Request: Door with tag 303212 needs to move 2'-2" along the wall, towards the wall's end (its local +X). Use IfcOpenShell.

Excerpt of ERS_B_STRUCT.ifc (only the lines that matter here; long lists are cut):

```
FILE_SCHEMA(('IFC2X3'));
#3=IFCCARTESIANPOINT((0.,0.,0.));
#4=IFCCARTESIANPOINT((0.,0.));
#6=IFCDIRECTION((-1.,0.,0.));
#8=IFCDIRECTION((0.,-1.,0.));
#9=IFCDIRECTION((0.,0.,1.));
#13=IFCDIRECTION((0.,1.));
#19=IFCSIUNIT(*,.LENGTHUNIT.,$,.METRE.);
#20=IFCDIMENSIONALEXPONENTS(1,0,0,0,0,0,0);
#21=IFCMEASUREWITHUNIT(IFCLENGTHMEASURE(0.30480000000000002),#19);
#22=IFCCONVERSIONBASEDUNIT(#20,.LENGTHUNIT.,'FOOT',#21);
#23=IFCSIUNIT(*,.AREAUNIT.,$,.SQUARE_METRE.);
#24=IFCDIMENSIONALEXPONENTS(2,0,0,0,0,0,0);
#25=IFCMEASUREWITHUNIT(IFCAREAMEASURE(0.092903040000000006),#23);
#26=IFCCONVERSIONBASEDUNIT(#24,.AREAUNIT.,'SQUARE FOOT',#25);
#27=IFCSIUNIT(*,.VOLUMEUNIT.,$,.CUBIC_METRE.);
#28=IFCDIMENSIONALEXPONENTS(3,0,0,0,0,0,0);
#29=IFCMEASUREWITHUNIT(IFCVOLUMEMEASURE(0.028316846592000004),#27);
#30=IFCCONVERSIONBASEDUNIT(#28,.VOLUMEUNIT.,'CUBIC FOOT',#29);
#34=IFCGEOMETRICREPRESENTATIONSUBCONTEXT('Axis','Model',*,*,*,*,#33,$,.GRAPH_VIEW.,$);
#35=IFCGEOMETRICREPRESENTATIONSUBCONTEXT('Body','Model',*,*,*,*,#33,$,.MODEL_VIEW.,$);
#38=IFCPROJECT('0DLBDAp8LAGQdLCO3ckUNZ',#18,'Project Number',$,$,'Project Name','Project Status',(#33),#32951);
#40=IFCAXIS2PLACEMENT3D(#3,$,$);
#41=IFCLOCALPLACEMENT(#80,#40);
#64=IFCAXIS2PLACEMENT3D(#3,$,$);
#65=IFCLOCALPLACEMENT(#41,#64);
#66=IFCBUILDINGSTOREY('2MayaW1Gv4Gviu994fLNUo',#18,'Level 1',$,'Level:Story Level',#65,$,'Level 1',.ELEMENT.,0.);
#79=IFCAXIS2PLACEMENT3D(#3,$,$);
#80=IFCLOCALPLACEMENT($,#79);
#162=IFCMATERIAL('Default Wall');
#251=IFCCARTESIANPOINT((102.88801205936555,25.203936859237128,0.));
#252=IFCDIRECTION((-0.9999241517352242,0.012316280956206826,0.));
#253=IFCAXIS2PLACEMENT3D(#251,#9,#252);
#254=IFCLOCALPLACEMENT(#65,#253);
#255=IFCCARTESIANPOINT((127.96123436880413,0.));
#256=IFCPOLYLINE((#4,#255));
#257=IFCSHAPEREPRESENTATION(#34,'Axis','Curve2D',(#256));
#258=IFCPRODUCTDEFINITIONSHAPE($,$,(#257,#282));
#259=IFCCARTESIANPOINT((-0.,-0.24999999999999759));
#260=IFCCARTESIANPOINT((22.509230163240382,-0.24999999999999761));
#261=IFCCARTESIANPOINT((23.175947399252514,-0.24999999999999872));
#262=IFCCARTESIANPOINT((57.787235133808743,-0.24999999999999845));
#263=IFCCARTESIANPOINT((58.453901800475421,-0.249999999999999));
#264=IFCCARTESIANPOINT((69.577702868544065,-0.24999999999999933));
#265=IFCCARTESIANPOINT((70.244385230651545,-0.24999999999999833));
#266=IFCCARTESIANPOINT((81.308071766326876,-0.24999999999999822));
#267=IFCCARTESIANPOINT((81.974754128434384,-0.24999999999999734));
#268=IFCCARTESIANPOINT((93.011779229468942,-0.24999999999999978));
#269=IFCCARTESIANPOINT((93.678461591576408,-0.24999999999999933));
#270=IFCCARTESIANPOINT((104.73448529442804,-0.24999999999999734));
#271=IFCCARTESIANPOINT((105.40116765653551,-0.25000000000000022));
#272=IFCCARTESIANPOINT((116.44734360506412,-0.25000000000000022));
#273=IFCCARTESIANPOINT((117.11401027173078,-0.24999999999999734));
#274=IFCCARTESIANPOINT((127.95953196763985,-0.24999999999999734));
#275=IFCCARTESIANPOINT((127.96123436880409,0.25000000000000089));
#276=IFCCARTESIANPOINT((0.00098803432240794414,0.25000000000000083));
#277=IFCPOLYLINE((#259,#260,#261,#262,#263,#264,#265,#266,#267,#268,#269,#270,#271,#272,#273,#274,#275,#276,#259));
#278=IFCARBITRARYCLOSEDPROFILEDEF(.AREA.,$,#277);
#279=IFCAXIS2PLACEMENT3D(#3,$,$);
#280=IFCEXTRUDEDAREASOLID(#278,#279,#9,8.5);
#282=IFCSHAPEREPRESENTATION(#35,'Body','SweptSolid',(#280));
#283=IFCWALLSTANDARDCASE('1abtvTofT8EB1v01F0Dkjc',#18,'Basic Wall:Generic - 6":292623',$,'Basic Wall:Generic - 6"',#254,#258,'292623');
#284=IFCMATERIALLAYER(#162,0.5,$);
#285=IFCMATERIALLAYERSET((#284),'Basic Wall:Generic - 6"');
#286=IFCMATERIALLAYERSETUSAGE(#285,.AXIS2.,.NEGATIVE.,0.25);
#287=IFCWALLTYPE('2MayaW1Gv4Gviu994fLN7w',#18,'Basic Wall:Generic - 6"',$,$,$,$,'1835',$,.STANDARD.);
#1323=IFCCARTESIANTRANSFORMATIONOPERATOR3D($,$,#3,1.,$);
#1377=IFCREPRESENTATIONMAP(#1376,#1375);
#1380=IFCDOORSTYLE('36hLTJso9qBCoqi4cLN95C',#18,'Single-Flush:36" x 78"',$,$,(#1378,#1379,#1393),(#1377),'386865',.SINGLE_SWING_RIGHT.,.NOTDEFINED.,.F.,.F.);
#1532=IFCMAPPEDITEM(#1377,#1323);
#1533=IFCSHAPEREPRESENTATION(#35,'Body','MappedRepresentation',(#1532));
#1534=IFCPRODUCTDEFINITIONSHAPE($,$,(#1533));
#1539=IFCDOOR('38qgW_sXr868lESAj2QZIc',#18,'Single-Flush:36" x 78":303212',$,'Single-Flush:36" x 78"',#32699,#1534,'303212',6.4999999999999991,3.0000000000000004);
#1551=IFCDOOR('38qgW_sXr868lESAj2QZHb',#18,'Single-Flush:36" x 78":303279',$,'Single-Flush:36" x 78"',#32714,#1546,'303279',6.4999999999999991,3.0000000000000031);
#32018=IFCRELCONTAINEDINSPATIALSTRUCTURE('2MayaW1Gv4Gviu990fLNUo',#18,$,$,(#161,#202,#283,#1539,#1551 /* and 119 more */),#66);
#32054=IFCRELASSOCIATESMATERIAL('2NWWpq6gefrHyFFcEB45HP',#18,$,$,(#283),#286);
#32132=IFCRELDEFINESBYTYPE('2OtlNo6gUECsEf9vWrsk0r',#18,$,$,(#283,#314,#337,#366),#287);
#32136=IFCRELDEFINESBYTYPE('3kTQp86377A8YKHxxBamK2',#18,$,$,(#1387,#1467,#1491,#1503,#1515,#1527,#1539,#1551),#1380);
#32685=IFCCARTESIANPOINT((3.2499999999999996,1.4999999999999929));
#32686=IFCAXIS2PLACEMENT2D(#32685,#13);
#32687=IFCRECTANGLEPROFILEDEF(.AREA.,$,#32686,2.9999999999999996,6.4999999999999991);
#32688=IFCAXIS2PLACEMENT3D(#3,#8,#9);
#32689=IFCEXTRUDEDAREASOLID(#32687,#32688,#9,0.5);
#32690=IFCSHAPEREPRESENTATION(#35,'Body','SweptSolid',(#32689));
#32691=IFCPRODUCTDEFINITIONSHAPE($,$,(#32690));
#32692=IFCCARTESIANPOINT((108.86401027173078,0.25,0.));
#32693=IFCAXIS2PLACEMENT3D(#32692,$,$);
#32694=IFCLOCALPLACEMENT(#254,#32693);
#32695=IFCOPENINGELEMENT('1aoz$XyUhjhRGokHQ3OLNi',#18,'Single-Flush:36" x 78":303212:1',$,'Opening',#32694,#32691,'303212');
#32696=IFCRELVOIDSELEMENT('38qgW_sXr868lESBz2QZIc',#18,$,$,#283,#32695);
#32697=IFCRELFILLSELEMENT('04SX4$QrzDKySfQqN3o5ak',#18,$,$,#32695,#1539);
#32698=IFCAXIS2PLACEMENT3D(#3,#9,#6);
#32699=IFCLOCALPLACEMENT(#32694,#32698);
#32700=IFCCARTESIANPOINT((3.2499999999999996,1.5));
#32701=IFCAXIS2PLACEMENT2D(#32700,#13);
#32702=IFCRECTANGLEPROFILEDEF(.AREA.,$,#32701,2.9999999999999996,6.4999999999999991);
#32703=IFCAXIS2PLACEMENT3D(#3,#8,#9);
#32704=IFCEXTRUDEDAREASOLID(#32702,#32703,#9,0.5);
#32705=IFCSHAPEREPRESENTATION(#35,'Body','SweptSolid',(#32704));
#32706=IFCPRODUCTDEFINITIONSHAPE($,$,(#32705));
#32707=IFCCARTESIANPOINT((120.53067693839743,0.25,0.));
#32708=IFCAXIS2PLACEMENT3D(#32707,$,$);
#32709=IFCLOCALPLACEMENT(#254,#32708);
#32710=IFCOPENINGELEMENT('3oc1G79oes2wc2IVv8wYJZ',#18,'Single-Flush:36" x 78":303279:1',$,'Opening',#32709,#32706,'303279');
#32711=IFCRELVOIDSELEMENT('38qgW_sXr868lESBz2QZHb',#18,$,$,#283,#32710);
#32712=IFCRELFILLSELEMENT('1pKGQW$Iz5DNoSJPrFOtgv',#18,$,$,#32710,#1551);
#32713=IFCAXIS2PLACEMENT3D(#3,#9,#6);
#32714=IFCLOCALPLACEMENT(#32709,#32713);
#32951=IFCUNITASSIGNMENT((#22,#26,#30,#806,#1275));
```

```python
import ifcopenshell
import ifcopenshell.api.geometry
import ifcopenshell.util.placement
import ifcopenshell.util.unit

model = ifcopenshell.open("ERS_B_STRUCT.ifc")
unit_scale = ifcopenshell.util.unit.calculate_unit_scale(model)

door = model.by_guid("38qgW_sXr868lESAj2QZIc")
opening = door.FillsVoids[0].RelatingOpeningElement
wall = opening.VoidsElements[0].RelatingBuildingElement

wall_matrix = ifcopenshell.util.placement.get_local_placement(wall.ObjectPlacement)
shift = wall_matrix[:3, 0] * 26 * 0.0254 / unit_scale
before = ifcopenshell.util.placement.get_local_placement(door.ObjectPlacement)[:3, 3].copy()

# The door is placed relative to its opening, so it follows when the opening moves.
matrix = ifcopenshell.util.placement.get_local_placement(opening.ObjectPlacement)
matrix[:3, 3] += shift
ifcopenshell.api.geometry.edit_object_placement(
    model, product=opening, matrix=matrix, is_si=False, should_transform_children=True
)

after = ifcopenshell.util.placement.get_local_placement(door.ObjectPlacement)[:3, 3]
print("door moved by", (after - before).round(3) + 0.0)

model.write("ERS_B_STRUCT_edited.ifc")
```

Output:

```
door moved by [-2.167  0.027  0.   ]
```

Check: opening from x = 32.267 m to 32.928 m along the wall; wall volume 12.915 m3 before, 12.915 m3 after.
